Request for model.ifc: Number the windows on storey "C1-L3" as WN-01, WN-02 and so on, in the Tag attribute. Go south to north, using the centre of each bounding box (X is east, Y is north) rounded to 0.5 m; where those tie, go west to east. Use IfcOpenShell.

First a look at what the model holds.

```python
import ifcopenshell
import ifcopenshell.util.element
import ifcopenshell.util.placement

model = ifcopenshell.open("model.ifc")
print(model.schema)
storey = next(s for s in model.by_type("IfcBuildingStorey") if s.Name == "C1-L3")
windows = [e for e in ifcopenshell.util.element.get_decomposition(storey) if e.is_a("IfcWindow")]
for e in sorted(windows, key=lambda e: e.id()):
    origin = ifcopenshell.util.placement.get_local_placement(e.ObjectPlacement)[:3, 3]
    print(e.id(), e.Tag, e.Name, origin.round(2) + 0.0, sep=" | ")
```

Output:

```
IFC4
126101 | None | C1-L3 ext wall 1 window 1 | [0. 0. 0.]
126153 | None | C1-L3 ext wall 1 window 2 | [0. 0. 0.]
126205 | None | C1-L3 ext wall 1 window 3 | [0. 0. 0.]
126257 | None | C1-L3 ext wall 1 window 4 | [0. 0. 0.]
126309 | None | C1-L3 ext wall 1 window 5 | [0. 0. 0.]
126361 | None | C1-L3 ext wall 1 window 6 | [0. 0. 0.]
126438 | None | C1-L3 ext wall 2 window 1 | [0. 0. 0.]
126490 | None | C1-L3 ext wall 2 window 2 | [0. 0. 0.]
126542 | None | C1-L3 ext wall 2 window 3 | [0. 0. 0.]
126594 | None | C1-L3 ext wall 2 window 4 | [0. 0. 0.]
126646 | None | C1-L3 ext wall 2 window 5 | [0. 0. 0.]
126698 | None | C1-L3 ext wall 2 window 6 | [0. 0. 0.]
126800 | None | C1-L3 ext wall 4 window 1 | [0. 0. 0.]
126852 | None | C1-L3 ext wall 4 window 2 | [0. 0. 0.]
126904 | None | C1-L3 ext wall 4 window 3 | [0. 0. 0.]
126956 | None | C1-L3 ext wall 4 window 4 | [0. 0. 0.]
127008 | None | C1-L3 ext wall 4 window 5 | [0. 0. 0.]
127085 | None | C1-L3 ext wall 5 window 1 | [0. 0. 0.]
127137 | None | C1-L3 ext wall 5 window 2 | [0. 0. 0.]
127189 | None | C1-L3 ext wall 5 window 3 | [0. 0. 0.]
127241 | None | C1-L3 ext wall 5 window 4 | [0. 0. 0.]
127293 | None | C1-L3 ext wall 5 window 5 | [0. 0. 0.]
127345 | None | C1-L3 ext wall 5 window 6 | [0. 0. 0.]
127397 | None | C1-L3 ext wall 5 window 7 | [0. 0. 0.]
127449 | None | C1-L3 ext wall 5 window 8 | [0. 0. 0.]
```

```python
import ifcopenshell
import ifcopenshell.geom
import ifcopenshell.util.element
import ifcopenshell.util.shape

model = ifcopenshell.open("model.ifc")
settings = ifcopenshell.geom.settings()
settings.set("use-world-coords", True)


def centre(element):
    shape = ifcopenshell.geom.create_shape(settings, element)
    return ifcopenshell.util.shape.get_bbox_centroid(shape.geometry)


storey = next(s for s in model.by_type("IfcBuildingStorey") if s.Name == "C1-L3")
windows = [e for e in ifcopenshell.util.element.get_decomposition(storey) if e.is_a("IfcWindow")]

# Insertion points can sit at a corner or the storey origin, so sort by the geometry (in metres).
centres = {e: centre(e) for e in windows}
windows.sort(key=lambda e: (round(centres[e][1] / 0.5), centres[e][0]))

for i, e in enumerate(windows, start=1):
    number = f"WN-{i:02d}"
    e.Tag = number
    print(e.id(), number)

model.write("model_edited.ifc")
```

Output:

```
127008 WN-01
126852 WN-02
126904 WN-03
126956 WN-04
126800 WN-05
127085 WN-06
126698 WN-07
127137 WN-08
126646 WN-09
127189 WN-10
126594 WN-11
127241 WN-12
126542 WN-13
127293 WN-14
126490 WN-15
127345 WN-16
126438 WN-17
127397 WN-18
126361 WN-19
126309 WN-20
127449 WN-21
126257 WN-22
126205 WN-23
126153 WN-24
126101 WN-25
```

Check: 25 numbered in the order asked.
